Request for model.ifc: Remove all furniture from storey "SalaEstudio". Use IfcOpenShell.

First a look at what the model holds.

```python
import ifcopenshell
import ifcopenshell.util.element

model = ifcopenshell.open("model.ifc")
print(model.schema)
storey = next(s for s in model.by_type("IfcBuildingStorey") if s.Name == "SalaEstudio")
furniture = [e for e in ifcopenshell.util.element.get_decomposition(storey) if e.is_a("IfcFurnishingElement")]
seen = {}
for e in furniture:
    element_type = ifcopenshell.util.element.get_type(e)
    name = element_type.Name if element_type not in (None, e) else None
    seen[name] = seen.get(name, 0) + 1
for name, count in sorted(seen.items(), key=str):
    print(count, "x", name)
```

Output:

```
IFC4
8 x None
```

```python
import ifcopenshell
import ifcopenshell.api.root
import ifcopenshell.util.element

model = ifcopenshell.open("model.ifc")

storey = next(s for s in model.by_type("IfcBuildingStorey") if s.Name == "SalaEstudio")
furniture = [e for e in ifcopenshell.util.element.get_decomposition(storey) if e.is_a("IfcFurnishingElement")]

for e in furniture:
    ifcopenshell.api.root.remove_product(model, product=e)
print(len(furniture), "removed")

model.write("model_v2.ifc")
```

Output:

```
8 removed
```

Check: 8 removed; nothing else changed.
